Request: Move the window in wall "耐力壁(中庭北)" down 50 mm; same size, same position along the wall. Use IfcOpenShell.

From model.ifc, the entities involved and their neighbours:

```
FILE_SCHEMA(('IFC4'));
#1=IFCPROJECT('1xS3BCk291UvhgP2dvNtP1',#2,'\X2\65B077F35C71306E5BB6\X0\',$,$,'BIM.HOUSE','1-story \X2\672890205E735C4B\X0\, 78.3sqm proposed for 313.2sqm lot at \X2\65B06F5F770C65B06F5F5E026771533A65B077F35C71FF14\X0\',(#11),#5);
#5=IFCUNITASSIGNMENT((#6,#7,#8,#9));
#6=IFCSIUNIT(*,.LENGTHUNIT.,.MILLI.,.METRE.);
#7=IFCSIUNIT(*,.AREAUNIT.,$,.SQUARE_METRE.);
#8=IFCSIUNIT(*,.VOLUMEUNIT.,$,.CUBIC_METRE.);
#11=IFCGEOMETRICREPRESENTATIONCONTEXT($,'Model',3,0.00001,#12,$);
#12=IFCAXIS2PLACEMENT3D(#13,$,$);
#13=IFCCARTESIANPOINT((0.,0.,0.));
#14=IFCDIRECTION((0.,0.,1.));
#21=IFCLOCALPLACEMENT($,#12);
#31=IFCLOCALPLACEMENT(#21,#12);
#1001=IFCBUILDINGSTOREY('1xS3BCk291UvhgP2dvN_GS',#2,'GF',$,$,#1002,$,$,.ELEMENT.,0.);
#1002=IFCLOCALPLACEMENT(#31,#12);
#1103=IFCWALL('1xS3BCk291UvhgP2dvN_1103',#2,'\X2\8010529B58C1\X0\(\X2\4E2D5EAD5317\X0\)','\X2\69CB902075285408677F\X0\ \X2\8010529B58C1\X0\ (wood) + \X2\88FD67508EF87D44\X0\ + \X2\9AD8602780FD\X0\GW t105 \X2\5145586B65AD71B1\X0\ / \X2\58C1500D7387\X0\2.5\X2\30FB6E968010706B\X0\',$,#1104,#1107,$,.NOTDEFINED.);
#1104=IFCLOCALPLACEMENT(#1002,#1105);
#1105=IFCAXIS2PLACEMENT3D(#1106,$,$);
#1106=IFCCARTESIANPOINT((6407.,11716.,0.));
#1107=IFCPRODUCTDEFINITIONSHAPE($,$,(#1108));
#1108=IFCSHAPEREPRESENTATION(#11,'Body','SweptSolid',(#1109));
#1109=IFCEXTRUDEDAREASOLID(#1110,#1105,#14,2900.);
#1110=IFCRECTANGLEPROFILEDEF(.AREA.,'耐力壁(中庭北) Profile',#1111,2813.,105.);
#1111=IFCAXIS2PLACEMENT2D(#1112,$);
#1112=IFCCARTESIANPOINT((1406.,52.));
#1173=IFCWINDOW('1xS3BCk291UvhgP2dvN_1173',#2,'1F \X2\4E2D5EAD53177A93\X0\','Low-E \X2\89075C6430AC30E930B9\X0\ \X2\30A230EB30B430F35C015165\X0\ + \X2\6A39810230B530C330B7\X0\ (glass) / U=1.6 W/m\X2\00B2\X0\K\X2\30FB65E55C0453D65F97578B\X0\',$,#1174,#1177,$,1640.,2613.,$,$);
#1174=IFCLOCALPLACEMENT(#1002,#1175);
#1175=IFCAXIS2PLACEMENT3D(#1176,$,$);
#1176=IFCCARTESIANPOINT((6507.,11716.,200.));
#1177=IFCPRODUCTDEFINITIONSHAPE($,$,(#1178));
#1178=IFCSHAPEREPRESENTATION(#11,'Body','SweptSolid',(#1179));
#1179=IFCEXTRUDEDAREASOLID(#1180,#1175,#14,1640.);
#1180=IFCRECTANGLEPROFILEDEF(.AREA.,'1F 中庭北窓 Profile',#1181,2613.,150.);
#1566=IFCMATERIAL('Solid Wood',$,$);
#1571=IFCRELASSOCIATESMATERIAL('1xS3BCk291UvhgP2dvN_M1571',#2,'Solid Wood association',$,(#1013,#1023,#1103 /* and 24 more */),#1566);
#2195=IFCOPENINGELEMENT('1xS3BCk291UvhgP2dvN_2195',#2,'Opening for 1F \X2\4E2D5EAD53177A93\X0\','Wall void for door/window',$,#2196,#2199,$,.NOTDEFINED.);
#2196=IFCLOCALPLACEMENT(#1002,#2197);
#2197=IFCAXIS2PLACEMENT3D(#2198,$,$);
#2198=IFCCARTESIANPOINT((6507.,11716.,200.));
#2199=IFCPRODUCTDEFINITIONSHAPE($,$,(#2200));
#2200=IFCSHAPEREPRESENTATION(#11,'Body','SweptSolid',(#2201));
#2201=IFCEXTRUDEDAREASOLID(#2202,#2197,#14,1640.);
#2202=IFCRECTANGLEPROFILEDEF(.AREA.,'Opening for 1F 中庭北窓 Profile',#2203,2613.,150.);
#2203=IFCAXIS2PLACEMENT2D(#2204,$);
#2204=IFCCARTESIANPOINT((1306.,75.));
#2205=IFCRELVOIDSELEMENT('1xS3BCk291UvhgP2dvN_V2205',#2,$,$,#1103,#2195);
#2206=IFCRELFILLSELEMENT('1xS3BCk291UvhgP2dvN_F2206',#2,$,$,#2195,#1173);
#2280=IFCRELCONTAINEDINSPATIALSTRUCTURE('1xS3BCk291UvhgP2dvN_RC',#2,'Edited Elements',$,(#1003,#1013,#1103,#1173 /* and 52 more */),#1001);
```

```python
import numpy as np
import ifcopenshell
import ifcopenshell.api.geometry
import ifcopenshell.util.placement
import ifcopenshell.util.unit

model = ifcopenshell.open("model.ifc")
unit_scale = ifcopenshell.util.unit.calculate_unit_scale(model)

window = model.by_guid("1xS3BCk291UvhgP2dvN_1173")
opening = window.FillsVoids[0].RelatingOpeningElement
dz = -0.05 / unit_scale

shift = np.array([0.0, 0.0, dz])
# The window is not placed relative to its opening, so move both.
for product in (opening, window):
    matrix = ifcopenshell.util.placement.get_local_placement(product.ObjectPlacement)
    matrix[:3, 3] += shift
    ifcopenshell.api.geometry.edit_object_placement(model, product=product, matrix=matrix, is_si=False)

print(f"moved by {dz * unit_scale:+.3f} m")

model.write("model-out.ifc")
```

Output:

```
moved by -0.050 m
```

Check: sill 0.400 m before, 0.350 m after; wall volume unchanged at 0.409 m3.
